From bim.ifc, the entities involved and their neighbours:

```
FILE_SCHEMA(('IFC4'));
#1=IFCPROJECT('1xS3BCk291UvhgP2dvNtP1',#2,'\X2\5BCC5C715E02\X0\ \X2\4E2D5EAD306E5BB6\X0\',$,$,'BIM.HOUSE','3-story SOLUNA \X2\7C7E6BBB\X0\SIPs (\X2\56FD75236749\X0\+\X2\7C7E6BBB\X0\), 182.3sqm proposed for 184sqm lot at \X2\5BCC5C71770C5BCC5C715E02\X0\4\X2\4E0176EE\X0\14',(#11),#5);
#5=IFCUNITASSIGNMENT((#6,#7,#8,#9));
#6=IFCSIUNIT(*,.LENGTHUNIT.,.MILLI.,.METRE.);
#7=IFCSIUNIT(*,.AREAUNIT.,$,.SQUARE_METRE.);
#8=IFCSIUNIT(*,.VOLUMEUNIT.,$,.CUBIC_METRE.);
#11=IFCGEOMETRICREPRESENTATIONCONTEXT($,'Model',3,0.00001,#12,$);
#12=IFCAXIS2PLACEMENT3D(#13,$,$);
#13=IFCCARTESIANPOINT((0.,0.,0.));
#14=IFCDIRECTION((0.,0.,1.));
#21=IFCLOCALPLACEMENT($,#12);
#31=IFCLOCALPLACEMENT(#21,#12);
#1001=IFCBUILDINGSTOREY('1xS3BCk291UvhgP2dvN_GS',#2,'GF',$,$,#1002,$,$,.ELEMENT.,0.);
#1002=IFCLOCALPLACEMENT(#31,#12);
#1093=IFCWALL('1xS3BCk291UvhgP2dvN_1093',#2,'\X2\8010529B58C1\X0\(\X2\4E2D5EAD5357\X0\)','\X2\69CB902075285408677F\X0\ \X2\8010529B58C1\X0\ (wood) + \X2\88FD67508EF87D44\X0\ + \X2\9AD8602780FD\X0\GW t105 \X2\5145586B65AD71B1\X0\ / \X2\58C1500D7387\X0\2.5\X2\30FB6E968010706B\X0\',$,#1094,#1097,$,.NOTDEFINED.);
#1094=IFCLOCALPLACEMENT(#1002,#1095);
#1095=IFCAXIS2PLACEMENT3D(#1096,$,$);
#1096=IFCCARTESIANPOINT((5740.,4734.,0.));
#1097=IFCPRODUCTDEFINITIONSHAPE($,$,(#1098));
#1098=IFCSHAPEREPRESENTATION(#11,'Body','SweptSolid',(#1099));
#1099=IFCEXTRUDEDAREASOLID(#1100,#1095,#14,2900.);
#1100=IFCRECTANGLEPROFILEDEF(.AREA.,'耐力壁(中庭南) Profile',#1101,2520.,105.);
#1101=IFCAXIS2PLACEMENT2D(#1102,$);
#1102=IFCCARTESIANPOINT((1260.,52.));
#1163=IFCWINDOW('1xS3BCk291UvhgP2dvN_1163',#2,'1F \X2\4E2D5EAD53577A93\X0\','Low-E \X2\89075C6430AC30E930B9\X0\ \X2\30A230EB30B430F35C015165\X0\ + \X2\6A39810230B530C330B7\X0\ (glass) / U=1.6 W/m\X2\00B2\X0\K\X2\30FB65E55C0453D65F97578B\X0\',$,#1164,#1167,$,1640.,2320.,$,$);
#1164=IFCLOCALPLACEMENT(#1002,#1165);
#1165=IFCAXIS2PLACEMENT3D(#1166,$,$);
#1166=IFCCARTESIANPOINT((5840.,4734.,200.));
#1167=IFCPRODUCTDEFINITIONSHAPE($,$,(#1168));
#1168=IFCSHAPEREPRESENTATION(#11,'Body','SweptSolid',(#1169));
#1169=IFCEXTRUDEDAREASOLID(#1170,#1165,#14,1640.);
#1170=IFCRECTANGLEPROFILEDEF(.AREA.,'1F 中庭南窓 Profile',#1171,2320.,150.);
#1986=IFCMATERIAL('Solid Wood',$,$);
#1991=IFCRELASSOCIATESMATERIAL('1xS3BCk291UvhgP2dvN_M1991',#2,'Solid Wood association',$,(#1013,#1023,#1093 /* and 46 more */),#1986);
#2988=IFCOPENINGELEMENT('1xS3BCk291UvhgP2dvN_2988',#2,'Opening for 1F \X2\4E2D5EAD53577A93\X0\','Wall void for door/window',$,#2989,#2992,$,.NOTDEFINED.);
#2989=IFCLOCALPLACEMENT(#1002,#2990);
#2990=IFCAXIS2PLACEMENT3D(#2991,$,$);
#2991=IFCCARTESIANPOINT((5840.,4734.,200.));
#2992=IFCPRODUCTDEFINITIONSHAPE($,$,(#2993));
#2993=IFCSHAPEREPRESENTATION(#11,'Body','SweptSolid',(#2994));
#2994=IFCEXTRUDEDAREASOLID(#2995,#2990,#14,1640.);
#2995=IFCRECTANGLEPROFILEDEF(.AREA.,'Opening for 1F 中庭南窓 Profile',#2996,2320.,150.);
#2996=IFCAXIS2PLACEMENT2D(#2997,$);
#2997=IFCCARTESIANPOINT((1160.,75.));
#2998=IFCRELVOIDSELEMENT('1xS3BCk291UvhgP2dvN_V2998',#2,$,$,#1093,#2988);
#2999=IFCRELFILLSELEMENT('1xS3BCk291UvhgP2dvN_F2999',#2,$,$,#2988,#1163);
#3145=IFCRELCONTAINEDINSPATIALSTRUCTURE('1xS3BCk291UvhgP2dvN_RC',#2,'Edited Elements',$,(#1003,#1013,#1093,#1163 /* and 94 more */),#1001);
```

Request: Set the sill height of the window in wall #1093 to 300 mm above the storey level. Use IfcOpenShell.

```python
import numpy as np
import ifcopenshell
import ifcopenshell.api.geometry
import ifcopenshell.geom
import ifcopenshell.util.element
import ifcopenshell.util.placement
import ifcopenshell.util.shape
import ifcopenshell.util.unit

model = ifcopenshell.open("bim.ifc")
unit_scale = ifcopenshell.util.unit.calculate_unit_scale(model)

window = model.by_guid("1xS3BCk291UvhgP2dvN_1163")
opening = window.FillsVoids[0].RelatingOpeningElement
storey = ifcopenshell.util.element.get_container(window, ifc_class="IfcBuildingStorey")
level = ifcopenshell.util.placement.get_local_placement(storey.ObjectPlacement)[2, 3]

# The opening's origin need not be at the sill, so measure its lowest point.
shape = ifcopenshell.geom.create_shape(ifcopenshell.geom.settings(), opening)
bottom = ifcopenshell.util.shape.get_shape_bottom_elevation(shape, shape.geometry) / unit_scale
dz = level + 300.0 - bottom

shift = np.array([0.0, 0.0, dz])
# The window is not placed relative to its opening, so move both.
for product in (opening, window):
    matrix = ifcopenshell.util.placement.get_local_placement(product.ObjectPlacement)
    matrix[:3, 3] += shift
    ifcopenshell.api.geometry.edit_object_placement(model, product=product, matrix=matrix, is_si=False)

print(f"moved by {dz * unit_scale:+.3f} m")

model.write("bim-out.ifc")
```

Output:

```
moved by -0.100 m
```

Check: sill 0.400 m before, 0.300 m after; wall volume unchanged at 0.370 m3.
